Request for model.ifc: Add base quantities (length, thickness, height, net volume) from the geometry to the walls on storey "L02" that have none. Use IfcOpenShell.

First a look at what the model holds.

```python
import ifcopenshell
import ifcopenshell.util.element
import ifcopenshell.util.unit

model = ifcopenshell.open("model.ifc")
print(model.schema)
for unit_type in ("LENGTHUNIT", "AREAUNIT", "VOLUMEUNIT"):
    print(unit_type, ifcopenshell.util.unit.calculate_unit_scale(model, unit_type))
storey = next(s for s in model.by_type("IfcBuildingStorey") if s.Name == "L02")
walls = [e for e in ifcopenshell.util.element.get_decomposition(storey) if e.is_a("IfcWall")]
for e in sorted(walls, key=lambda e: e.id()):
    print(e.id(), e.is_a(), e.Name, list(ifcopenshell.util.element.get_psets(e, qtos_only=True)), sep=" | ")
```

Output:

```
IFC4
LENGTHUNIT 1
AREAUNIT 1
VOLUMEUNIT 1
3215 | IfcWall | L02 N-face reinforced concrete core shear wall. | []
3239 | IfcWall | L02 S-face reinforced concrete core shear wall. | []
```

```python
import ifcopenshell
import ifcopenshell.api.pset
import ifcopenshell.geom
import ifcopenshell.util.element
import ifcopenshell.util.shape
import ifcopenshell.util.unit

model = ifcopenshell.open("model.ifc")
unit_scale = ifcopenshell.util.unit.calculate_unit_scale(model)
volume_scale = ifcopenshell.util.unit.calculate_unit_scale(model, "VOLUMEUNIT")
settings = ifcopenshell.geom.settings()

storey = next(s for s in model.by_type("IfcBuildingStorey") if s.Name == "L02")
walls = [e for e in ifcopenshell.util.element.get_decomposition(storey) if e.is_a("IfcWall")]

for e in sorted(walls, key=lambda e: e.id()):
    if ifcopenshell.util.element.get_psets(e, qtos_only=True, should_inherit=False):
        continue
    # Geometry comes back in metres, in the element's own axes.
    shape = ifcopenshell.geom.create_shape(settings, e)
    values = {
        "Length": ifcopenshell.util.shape.get_x(shape.geometry) / unit_scale,
        "Width": ifcopenshell.util.shape.get_y(shape.geometry) / unit_scale,
        "Height": ifcopenshell.util.shape.get_z(shape.geometry) / unit_scale,
        "NetVolume": ifcopenshell.util.shape.get_volume(shape.geometry) / volume_scale,
    }
    qto = ifcopenshell.api.pset.add_qto(model, product=e, name="Qto_WallBaseQuantities")
    ifcopenshell.api.pset.edit_qto(model, qto=qto, properties=values)
    print(e.id(), {k: round(v, 3) for k, v in values.items()})

model.write("model-out.ifc")
```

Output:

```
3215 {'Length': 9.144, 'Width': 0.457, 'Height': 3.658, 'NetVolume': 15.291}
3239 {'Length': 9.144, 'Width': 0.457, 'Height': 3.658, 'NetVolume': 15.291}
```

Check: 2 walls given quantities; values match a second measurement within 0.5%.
